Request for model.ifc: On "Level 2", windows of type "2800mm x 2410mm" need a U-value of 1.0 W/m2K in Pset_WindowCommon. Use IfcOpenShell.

First a look at what the model holds.

```python
import ifcopenshell
import ifcopenshell.util.element

model = ifcopenshell.open("model.ifc")
print(model.schema)
storey = next(s for s in model.by_type("IfcBuildingStorey") if s.Name == "Level 2")
windows = [e for e in ifcopenshell.util.element.get_decomposition(storey) if e.is_a("IfcWindow")]
seen = {}
for e in windows:
    element_type = ifcopenshell.util.element.get_type(e)
    key = (element_type.Name if element_type != e and element_type else None, ifcopenshell.util.element.get_pset(e, "Pset_WindowCommon", "ThermalTransmittance"))
    seen[key] = seen.get(key, 0) + 1
for (name, value), count in sorted(seen.items(), key=str):
    print(count, "x", name, "|", value)
```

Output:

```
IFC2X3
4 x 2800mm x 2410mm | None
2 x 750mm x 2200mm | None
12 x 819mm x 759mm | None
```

```python
import ifcopenshell
import ifcopenshell.api.pset
import ifcopenshell.util.element

model = ifcopenshell.open("model.ifc")

storey = next(s for s in model.by_type("IfcBuildingStorey") if s.Name == "Level 2")
windows = [e for e in ifcopenshell.util.element.get_decomposition(storey) if e.is_a("IfcWindow")]

count = 0
for e in windows:
    element_type = ifcopenshell.util.element.get_type(e)
    if element_type in (None, e) or element_type.Name != "2800mm x 2410mm":
        continue
    # add_pset returns the element's existing set when there is one.
    pset = ifcopenshell.api.pset.add_pset(model, product=e, name="Pset_WindowCommon")
    ifcopenshell.api.pset.edit_pset(model, pset=pset, properties={"ThermalTransmittance": 1.0})
    count += 1

print(count, "windows updated")

model.write("model_edited.ifc")
```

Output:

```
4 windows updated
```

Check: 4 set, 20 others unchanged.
